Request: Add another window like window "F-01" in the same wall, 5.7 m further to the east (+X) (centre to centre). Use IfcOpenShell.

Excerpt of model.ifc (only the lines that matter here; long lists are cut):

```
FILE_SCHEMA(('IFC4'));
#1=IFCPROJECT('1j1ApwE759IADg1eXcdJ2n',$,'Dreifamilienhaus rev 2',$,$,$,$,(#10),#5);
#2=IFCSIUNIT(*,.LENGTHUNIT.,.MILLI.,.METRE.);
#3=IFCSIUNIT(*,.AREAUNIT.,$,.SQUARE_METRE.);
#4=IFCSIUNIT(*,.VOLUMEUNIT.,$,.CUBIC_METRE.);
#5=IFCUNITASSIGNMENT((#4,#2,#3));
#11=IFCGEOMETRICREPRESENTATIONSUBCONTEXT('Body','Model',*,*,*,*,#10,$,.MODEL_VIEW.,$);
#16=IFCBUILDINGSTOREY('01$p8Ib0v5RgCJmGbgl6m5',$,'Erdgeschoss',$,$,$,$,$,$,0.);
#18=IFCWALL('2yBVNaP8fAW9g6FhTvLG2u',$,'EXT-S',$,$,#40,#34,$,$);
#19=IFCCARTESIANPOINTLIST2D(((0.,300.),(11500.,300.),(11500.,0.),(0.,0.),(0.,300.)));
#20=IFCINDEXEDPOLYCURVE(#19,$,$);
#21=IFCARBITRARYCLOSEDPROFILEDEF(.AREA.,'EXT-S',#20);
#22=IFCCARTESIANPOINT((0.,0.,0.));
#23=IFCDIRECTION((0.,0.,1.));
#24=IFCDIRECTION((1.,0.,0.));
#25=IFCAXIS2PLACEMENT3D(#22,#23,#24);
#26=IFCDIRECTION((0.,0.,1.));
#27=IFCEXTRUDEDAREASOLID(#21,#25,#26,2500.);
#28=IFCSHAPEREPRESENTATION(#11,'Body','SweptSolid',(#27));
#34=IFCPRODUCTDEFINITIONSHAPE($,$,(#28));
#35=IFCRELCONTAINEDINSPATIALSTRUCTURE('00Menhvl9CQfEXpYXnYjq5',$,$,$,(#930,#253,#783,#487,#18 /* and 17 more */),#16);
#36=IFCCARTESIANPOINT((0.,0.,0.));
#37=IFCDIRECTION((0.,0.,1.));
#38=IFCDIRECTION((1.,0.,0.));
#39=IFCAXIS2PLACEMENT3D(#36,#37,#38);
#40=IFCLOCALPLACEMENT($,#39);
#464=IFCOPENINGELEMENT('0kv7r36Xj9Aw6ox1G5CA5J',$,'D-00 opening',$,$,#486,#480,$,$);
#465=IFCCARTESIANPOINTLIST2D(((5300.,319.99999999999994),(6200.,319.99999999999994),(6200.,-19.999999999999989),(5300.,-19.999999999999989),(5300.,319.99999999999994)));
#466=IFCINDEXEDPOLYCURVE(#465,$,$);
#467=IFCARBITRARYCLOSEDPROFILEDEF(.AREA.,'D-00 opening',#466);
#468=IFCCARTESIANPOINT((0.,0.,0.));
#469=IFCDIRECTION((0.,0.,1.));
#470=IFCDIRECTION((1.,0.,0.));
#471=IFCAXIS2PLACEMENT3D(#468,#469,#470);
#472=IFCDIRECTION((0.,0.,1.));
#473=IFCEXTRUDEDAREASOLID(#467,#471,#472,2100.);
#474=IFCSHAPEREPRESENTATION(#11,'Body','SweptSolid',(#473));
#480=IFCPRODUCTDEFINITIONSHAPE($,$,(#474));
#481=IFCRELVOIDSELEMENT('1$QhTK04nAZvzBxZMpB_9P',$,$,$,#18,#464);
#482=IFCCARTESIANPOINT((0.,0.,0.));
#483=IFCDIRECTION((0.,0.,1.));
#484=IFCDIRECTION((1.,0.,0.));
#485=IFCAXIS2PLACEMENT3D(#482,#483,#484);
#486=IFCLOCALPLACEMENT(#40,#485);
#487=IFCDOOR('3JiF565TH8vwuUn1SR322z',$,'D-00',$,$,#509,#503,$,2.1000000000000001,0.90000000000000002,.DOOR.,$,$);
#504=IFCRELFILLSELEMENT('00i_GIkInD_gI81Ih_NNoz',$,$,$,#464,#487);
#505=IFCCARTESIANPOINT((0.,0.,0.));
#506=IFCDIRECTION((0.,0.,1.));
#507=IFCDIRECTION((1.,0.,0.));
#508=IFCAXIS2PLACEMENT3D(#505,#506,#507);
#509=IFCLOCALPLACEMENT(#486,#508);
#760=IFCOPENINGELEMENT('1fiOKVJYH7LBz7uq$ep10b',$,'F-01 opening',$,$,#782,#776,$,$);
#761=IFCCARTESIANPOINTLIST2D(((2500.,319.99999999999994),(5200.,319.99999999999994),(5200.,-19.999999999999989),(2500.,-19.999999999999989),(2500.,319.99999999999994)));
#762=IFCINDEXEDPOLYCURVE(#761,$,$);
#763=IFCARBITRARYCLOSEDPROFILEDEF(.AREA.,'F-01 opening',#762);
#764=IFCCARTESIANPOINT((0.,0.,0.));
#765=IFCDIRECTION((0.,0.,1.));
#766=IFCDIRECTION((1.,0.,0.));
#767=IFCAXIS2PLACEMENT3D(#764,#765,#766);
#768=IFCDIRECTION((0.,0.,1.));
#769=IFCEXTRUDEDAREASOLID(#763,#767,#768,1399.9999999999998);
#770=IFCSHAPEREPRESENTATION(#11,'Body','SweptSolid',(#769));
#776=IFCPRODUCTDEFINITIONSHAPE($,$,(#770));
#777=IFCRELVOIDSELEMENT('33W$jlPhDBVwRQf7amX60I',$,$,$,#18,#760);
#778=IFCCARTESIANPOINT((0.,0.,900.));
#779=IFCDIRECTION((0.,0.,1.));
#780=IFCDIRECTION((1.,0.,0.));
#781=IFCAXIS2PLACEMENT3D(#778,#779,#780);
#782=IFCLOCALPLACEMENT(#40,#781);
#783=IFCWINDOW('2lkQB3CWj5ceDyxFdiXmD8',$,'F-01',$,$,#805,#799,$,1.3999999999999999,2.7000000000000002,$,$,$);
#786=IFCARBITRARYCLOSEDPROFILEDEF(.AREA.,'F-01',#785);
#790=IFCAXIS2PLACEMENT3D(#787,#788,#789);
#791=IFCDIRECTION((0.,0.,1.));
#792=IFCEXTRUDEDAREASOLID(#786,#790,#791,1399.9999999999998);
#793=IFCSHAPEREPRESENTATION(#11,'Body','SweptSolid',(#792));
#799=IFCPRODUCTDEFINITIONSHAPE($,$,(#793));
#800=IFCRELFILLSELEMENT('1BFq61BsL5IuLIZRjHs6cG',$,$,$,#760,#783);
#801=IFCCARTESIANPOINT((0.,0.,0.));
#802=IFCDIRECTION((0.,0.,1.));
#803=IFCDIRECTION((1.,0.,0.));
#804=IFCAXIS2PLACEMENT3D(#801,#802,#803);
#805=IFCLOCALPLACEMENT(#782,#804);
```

```python
import ifcopenshell
import ifcopenshell.api.feature
import ifcopenshell.api.geometry
import ifcopenshell.api.root
import ifcopenshell.geom
import ifcopenshell.util.element
import ifcopenshell.util.placement
import ifcopenshell.util.shape

model = ifcopenshell.open("model.ifc")
settings = ifcopenshell.geom.settings()


def volume(element):
    """Net volume in cubic metres, openings subtracted."""
    shape = ifcopenshell.geom.create_shape(settings, element)
    return ifcopenshell.util.shape.get_volume(shape.geometry)


window = model.by_guid("2lkQB3CWj5ceDyxFdiXmD8")
opening = window.FillsVoids[0].RelatingOpeningElement
wall = opening.VoidsElements[0].RelatingBuildingElement
before = volume(wall)
shift = ifcopenshell.util.placement.get_local_placement(wall.ObjectPlacement)[:3, 0] * 5700.0

# copy_class copies the void relationship, type, container and properties, but no geometry.
new_opening = ifcopenshell.api.root.copy_class(model, product=opening)
new_opening.Representation = ifcopenshell.util.element.copy_deep(
    model, opening.Representation, exclude=["IfcGeometricRepresentationContext", "IfcRepresentationMap"]
)
new_window = ifcopenshell.api.root.copy_class(model, product=window)
new_window.Representation = ifcopenshell.util.element.copy_deep(
    model, window.Representation, exclude=["IfcGeometricRepresentationContext", "IfcRepresentationMap"]
)
ifcopenshell.api.feature.add_filling(model, opening=new_opening, element=new_window)

for old, new in ((opening, new_opening), (window, new_window)):
    matrix = ifcopenshell.util.placement.get_local_placement(old.ObjectPlacement)
    matrix[:3, 3] += shift
    ifcopenshell.api.geometry.edit_object_placement(model, product=new, matrix=matrix, is_si=False)

after = volume(wall)

print(f"wall volume {before:.3f} -> {after:.3f} m3")

model.write("model_edited.ifc")
```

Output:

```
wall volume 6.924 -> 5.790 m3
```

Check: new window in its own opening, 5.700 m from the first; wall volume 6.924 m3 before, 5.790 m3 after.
